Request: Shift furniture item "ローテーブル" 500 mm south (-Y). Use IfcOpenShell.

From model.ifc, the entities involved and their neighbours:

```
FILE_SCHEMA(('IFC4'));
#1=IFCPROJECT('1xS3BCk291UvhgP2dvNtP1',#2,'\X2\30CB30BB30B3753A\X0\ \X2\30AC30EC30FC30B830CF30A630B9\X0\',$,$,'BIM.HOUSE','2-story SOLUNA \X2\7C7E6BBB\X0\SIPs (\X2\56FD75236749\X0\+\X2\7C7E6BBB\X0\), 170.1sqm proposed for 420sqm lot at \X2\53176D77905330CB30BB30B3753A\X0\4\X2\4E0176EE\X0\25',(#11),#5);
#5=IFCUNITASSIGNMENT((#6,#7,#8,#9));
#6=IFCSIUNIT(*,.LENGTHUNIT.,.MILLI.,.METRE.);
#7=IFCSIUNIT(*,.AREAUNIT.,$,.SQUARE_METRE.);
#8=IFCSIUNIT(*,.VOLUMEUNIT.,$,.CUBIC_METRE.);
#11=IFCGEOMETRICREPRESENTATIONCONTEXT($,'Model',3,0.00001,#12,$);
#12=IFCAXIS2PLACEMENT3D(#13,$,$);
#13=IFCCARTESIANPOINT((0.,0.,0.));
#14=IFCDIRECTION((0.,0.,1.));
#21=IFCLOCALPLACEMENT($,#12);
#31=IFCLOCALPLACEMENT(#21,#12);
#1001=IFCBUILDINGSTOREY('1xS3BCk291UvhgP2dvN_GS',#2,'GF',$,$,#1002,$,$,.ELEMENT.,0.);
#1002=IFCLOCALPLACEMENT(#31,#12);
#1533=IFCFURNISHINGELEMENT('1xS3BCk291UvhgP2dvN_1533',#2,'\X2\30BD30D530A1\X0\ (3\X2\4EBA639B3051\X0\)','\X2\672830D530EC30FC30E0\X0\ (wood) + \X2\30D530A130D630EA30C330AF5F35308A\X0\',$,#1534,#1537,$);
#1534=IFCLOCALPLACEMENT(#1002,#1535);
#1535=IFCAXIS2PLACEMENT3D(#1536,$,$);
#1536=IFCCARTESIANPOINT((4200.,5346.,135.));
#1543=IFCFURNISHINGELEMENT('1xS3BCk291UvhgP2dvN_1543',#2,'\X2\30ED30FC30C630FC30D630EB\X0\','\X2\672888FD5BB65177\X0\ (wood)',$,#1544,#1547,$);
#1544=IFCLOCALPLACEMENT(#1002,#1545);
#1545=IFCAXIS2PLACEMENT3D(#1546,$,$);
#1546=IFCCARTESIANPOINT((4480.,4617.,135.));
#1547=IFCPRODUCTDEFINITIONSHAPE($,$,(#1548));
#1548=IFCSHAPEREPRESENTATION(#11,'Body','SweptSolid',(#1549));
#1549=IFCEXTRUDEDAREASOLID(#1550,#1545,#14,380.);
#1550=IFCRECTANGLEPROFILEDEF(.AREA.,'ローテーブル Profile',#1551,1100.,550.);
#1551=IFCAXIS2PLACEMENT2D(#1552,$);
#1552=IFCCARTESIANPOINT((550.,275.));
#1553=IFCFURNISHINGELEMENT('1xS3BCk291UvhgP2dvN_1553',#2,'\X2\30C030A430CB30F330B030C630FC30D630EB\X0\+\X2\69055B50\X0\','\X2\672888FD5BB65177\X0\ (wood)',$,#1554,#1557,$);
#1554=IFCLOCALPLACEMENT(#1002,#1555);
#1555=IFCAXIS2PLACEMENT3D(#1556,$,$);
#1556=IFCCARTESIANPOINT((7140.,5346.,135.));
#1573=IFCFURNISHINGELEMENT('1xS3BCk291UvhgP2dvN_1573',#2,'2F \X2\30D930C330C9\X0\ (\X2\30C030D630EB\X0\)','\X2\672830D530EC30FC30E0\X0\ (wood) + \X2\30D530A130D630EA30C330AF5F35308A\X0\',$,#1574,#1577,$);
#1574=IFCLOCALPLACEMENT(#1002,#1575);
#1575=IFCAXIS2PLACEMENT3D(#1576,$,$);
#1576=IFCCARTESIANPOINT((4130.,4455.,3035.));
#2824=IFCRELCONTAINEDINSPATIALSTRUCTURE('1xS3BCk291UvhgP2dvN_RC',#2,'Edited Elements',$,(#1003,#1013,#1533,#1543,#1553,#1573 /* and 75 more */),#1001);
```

```python
import ifcopenshell
import ifcopenshell.api.geometry
import ifcopenshell.util.placement
import ifcopenshell.util.unit

model = ifcopenshell.open("model.ifc")
unit_scale = ifcopenshell.util.unit.calculate_unit_scale(model)

item = model.by_guid("1xS3BCk291UvhgP2dvN_1543")
matrix = ifcopenshell.util.placement.get_local_placement(item.ObjectPlacement)
matrix[1, 3] -= 0.5 / unit_scale
ifcopenshell.api.geometry.edit_object_placement(model, product=item, matrix=matrix, is_si=False)

print(ifcopenshell.util.placement.get_local_placement(item.ObjectPlacement).round(3) + 0.0)

model.write("model_edited.ifc")
```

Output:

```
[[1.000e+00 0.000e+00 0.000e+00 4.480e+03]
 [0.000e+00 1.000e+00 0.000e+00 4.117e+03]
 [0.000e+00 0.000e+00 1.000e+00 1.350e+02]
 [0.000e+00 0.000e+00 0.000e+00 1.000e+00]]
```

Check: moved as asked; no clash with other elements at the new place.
